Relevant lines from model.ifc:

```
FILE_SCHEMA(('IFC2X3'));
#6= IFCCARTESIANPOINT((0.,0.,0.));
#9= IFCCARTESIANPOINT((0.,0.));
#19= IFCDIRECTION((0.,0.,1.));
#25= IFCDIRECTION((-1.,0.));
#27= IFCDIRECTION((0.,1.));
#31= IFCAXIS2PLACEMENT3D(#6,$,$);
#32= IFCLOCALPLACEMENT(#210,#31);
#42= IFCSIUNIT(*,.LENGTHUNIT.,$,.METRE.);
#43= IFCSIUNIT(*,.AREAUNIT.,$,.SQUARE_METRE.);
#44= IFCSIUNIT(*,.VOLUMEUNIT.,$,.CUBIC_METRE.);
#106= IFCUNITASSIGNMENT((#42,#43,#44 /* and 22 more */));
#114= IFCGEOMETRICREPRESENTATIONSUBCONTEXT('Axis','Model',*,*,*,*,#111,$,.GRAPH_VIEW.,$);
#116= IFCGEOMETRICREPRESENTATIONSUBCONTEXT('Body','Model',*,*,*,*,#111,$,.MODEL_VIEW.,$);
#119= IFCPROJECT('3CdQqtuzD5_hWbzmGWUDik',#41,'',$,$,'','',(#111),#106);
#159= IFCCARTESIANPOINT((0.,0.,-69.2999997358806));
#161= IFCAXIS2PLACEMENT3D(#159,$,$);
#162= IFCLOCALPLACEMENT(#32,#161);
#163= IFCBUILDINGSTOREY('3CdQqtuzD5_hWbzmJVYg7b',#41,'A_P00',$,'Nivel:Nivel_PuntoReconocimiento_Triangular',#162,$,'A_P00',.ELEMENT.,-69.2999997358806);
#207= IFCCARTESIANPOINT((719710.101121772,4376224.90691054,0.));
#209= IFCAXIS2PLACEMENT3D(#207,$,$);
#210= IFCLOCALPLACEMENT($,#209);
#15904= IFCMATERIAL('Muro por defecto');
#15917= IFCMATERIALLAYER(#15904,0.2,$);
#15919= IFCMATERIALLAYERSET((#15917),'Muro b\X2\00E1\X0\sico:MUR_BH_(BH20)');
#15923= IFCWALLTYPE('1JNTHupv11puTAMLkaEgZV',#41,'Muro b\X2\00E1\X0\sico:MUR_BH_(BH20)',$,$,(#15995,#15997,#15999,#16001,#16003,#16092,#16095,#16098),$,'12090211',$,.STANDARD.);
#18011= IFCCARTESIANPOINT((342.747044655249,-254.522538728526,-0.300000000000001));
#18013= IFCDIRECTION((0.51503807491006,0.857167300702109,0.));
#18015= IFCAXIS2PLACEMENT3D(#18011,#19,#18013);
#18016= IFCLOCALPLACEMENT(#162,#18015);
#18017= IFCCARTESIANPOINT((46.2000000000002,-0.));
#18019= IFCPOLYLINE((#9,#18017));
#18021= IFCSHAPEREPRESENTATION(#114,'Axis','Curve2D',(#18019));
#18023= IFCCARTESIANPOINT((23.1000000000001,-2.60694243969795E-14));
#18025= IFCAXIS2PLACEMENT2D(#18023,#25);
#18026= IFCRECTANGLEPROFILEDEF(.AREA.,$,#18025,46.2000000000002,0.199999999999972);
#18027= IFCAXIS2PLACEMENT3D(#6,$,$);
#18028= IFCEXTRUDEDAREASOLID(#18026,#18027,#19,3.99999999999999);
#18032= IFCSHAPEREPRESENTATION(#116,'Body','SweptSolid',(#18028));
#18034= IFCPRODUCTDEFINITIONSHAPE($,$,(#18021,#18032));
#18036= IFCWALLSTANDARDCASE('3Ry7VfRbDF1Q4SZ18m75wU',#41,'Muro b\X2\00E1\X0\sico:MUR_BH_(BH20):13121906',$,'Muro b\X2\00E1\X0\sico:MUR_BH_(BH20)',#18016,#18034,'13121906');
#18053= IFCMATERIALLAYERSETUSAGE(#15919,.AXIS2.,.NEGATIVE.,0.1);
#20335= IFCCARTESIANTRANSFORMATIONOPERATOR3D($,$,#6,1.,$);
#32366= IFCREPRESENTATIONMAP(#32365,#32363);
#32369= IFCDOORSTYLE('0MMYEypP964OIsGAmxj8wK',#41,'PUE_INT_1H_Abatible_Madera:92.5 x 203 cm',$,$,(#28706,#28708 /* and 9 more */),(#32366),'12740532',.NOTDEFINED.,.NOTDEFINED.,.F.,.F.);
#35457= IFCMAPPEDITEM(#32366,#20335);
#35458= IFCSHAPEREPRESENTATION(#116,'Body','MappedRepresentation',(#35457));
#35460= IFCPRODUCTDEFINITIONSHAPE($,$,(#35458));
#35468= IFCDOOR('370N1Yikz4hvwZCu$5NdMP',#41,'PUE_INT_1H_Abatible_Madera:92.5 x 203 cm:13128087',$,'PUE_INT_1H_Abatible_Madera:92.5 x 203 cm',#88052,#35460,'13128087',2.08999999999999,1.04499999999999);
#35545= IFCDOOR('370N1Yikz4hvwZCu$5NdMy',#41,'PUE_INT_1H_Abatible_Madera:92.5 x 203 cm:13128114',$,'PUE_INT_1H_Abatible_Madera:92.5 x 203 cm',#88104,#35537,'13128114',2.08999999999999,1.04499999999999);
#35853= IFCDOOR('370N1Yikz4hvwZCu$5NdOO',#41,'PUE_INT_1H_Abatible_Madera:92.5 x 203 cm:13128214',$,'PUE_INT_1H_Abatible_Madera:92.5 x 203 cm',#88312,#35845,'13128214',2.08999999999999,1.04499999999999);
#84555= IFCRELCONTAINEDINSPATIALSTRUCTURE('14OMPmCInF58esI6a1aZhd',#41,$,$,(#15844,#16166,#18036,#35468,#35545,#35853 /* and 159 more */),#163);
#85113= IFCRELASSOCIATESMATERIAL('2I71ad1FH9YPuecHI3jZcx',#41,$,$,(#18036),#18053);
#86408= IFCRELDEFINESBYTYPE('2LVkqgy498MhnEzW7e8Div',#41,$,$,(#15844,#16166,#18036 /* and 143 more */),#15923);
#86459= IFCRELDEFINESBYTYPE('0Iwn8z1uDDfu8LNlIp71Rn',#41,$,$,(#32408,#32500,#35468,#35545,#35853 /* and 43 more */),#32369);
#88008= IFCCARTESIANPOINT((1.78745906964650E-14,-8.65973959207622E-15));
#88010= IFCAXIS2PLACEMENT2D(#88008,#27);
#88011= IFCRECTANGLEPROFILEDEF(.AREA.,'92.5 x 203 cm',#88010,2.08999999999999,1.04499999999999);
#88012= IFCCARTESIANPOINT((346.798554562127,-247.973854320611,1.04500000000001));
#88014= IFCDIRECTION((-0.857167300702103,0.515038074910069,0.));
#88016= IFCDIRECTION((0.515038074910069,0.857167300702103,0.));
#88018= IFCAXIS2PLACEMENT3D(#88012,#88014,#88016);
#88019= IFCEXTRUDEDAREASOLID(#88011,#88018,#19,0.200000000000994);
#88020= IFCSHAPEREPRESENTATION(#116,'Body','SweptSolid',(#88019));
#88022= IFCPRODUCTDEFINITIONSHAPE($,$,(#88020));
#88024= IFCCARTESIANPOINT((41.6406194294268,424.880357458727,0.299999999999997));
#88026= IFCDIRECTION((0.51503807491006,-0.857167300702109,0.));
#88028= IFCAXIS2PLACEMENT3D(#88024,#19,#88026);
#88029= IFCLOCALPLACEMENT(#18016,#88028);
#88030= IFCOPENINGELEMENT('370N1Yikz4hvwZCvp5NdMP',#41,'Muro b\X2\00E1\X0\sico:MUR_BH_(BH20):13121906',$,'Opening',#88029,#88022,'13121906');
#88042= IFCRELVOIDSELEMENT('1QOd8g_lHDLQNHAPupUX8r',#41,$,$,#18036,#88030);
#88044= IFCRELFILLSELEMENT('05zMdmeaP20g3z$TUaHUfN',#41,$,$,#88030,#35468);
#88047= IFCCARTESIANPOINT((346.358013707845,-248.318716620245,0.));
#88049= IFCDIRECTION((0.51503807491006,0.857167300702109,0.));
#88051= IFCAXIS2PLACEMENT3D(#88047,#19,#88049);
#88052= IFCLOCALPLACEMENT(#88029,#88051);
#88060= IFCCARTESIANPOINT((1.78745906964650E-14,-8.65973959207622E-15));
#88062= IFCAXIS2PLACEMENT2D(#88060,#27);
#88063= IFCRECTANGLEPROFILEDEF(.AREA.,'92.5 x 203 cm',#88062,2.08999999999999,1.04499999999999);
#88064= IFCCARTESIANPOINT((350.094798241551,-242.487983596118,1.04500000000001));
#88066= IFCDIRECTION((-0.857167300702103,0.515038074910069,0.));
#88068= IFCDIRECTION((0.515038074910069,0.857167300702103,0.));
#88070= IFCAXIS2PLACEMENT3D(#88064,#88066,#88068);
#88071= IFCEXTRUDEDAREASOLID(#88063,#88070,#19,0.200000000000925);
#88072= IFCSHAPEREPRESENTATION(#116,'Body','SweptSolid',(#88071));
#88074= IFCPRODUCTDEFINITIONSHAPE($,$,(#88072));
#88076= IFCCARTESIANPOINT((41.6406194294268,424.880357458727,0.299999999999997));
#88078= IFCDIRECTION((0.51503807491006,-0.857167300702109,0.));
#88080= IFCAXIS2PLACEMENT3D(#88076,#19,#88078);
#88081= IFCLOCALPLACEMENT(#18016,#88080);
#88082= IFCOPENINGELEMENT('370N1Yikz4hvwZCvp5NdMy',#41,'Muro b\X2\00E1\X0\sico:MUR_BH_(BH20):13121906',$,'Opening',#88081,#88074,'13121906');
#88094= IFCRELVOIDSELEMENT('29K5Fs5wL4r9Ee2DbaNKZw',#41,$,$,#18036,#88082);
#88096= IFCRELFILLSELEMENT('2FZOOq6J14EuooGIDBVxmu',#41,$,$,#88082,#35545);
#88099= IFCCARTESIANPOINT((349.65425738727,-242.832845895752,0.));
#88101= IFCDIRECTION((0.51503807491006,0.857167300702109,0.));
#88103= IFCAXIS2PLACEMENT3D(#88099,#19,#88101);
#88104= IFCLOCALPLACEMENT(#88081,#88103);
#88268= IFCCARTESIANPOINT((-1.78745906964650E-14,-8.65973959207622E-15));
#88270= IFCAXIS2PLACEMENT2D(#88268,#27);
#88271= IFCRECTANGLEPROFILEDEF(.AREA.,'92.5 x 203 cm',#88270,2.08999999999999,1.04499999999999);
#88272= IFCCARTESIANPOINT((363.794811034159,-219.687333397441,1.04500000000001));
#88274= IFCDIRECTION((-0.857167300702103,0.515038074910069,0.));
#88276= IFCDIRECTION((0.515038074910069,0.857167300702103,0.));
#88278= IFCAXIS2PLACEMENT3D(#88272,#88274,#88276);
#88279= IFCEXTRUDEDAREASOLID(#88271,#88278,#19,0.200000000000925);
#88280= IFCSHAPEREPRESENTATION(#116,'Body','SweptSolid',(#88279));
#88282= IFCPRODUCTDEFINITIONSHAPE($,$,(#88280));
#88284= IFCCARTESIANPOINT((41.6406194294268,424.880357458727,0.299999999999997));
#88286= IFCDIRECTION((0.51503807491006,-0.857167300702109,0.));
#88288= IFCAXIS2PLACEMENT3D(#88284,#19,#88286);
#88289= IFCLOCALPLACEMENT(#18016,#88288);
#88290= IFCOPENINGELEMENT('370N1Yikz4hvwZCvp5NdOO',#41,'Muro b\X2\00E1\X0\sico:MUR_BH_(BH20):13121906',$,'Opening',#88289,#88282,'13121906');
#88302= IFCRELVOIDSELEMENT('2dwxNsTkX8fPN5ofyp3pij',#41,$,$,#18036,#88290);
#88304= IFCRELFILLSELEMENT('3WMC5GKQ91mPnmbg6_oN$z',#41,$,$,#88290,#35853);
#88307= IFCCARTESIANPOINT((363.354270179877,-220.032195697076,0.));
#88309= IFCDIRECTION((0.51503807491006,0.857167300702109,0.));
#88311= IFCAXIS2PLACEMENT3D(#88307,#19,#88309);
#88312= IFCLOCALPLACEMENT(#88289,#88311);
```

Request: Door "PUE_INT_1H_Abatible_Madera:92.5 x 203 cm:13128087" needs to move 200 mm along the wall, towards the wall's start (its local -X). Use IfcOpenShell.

```python
import ifcopenshell
import ifcopenshell.api.geometry
import ifcopenshell.util.placement
import ifcopenshell.util.unit

model = ifcopenshell.open("model.ifc")
unit_scale = ifcopenshell.util.unit.calculate_unit_scale(model)

door = model.by_guid("370N1Yikz4hvwZCu$5NdMP")
opening = door.FillsVoids[0].RelatingOpeningElement
wall = opening.VoidsElements[0].RelatingBuildingElement

wall_matrix = ifcopenshell.util.placement.get_local_placement(wall.ObjectPlacement)
shift = wall_matrix[:3, 0] * -0.2 / unit_scale
before = ifcopenshell.util.placement.get_local_placement(door.ObjectPlacement)[:3, 3].copy()

# The door is placed relative to its opening, so it follows when the opening moves.
matrix = ifcopenshell.util.placement.get_local_placement(opening.ObjectPlacement)
matrix[:3, 3] += shift
ifcopenshell.api.geometry.edit_object_placement(
    model, product=opening, matrix=matrix, is_si=False, should_transform_children=True
)

after = ifcopenshell.util.placement.get_local_placement(door.ObjectPlacement)[:3, 3]
print("door moved by", (after - before).round(3) + 0.0)

model.write("model-out.ifc")
```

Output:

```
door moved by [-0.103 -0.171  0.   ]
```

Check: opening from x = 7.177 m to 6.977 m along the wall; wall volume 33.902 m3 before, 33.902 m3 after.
